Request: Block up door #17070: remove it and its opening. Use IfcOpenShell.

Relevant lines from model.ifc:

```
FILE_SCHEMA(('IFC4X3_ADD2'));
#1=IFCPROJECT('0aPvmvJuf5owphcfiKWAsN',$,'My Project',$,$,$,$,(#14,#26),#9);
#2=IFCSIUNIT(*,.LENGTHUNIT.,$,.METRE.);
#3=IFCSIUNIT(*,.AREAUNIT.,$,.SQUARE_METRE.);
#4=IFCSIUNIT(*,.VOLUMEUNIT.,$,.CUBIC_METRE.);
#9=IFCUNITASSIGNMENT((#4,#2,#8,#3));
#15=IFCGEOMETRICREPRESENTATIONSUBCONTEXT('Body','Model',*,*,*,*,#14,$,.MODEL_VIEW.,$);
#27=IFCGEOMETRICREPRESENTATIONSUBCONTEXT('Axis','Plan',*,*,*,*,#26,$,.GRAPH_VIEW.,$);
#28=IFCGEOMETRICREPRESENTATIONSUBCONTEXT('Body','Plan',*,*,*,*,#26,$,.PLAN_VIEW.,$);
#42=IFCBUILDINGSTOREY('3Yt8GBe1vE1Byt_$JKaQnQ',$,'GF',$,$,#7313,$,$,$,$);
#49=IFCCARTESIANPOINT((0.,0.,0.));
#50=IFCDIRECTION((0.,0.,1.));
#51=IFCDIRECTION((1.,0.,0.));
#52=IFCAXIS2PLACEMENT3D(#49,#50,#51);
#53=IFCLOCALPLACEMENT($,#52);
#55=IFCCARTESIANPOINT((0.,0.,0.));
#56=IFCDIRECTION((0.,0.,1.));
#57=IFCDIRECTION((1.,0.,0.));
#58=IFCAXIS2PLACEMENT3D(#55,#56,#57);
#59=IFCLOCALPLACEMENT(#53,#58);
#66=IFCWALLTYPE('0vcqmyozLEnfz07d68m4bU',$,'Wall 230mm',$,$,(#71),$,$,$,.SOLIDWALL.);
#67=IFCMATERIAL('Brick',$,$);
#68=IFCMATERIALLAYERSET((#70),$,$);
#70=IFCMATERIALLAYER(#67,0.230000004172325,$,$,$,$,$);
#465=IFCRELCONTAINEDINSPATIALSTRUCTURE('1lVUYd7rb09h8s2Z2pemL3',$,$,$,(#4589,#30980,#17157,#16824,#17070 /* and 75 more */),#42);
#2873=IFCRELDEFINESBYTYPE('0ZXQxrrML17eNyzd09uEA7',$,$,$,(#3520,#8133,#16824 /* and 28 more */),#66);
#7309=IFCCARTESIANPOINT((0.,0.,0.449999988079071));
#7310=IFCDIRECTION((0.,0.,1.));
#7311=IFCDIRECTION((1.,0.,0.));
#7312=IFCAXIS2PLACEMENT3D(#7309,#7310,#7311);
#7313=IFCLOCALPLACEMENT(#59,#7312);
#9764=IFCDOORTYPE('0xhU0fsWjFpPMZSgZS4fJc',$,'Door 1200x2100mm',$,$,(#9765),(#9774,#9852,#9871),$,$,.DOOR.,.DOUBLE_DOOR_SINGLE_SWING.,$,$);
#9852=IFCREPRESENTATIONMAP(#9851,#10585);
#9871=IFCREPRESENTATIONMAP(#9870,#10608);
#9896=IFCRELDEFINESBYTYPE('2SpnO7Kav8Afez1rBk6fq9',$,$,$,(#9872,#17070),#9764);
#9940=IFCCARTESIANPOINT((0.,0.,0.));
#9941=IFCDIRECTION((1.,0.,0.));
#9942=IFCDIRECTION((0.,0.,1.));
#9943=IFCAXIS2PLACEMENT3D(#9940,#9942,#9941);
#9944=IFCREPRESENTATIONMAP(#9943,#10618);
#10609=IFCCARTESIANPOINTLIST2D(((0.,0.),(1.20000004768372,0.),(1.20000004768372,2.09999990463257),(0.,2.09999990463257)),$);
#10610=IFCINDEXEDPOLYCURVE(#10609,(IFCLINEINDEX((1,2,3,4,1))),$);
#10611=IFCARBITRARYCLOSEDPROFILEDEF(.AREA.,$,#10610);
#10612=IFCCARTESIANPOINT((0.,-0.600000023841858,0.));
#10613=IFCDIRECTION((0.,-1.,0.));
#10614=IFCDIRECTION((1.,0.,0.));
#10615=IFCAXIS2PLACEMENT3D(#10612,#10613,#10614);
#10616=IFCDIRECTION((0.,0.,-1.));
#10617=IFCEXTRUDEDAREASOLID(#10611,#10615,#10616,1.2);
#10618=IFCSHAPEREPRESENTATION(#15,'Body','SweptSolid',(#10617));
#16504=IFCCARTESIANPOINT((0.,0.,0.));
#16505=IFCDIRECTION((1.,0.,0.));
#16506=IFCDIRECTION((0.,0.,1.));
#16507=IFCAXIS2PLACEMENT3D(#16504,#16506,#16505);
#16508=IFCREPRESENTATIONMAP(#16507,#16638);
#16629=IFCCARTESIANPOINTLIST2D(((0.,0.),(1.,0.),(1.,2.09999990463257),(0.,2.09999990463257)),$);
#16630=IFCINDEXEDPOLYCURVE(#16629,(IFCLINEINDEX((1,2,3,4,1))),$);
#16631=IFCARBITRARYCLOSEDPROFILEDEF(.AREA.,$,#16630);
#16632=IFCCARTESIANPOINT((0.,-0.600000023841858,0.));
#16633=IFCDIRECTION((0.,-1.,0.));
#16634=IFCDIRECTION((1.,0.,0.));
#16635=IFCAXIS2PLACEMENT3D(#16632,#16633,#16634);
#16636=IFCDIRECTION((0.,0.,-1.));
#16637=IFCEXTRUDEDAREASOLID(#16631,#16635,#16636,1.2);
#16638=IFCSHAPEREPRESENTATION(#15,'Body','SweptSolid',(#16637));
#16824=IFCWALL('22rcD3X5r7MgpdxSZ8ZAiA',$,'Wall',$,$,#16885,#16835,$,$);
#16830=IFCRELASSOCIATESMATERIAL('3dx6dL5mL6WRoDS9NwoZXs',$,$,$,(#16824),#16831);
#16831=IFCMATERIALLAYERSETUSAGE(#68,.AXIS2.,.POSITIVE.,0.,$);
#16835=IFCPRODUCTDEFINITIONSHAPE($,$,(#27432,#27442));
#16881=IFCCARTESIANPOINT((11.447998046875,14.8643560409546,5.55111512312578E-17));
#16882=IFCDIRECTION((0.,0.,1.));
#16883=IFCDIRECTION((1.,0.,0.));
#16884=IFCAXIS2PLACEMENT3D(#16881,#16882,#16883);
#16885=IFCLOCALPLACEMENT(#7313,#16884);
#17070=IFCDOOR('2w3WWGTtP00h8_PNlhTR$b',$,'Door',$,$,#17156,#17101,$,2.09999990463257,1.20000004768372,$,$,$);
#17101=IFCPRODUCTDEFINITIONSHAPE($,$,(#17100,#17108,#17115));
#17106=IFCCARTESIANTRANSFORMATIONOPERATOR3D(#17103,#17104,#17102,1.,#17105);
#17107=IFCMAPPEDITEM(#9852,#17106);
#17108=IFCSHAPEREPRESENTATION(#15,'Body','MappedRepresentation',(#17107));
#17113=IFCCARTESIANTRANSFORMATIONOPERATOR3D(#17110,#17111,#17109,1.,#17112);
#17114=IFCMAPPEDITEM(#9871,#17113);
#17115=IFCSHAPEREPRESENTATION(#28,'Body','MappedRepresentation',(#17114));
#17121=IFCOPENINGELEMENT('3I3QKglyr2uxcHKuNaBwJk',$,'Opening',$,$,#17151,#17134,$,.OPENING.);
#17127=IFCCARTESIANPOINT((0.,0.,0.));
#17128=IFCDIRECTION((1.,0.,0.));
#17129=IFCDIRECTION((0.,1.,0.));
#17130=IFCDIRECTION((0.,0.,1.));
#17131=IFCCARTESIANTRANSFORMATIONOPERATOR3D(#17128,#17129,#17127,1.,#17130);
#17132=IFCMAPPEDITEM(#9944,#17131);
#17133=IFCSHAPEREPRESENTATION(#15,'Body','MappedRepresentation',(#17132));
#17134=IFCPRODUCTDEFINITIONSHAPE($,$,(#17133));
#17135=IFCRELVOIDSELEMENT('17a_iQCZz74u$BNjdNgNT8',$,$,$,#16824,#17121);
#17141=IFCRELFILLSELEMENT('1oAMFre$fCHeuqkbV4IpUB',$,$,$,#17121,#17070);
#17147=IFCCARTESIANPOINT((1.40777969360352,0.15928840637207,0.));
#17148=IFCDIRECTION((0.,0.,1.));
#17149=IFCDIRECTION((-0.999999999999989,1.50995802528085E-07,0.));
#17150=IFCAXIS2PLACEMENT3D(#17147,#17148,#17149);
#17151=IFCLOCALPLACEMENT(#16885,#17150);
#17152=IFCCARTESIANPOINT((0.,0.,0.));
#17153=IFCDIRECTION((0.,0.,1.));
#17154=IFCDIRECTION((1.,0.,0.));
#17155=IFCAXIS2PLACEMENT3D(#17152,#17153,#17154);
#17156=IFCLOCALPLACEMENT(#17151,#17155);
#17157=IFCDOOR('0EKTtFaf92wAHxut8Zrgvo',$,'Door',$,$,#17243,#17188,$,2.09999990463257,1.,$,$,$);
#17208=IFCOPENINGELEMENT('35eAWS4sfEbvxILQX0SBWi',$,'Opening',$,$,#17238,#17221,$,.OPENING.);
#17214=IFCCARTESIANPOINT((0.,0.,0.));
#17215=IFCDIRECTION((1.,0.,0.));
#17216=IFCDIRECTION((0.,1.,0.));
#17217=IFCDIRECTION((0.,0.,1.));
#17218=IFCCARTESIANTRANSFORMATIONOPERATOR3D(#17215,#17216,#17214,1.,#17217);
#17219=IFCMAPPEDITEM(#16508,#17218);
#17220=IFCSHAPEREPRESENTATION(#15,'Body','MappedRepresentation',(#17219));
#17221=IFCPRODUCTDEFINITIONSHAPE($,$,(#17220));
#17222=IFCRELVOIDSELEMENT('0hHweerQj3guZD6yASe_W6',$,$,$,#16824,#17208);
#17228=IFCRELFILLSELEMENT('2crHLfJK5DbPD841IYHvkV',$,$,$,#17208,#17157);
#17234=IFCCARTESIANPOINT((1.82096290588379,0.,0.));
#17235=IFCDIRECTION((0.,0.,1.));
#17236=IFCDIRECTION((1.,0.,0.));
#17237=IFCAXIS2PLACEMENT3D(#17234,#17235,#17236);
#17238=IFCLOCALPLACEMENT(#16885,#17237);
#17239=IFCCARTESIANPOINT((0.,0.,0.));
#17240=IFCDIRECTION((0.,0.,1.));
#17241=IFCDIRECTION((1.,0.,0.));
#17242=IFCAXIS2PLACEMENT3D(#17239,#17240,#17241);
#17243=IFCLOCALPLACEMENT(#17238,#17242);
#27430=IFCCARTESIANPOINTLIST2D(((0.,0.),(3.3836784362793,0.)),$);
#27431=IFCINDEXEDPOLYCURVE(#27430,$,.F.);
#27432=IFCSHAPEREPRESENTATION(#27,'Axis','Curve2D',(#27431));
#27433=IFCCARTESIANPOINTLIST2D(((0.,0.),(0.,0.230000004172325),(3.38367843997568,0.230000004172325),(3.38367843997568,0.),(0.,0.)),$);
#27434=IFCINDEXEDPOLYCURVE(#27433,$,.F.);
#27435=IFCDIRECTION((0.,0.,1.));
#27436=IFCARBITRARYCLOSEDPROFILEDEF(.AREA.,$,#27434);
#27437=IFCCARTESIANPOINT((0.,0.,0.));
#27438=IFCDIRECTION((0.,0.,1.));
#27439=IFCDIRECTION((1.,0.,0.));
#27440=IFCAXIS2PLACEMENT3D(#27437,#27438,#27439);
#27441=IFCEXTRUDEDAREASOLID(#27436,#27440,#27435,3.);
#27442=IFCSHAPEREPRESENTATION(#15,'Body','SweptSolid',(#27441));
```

```python
import ifcopenshell
import ifcopenshell.api.feature
import ifcopenshell.api.root
import ifcopenshell.geom
import ifcopenshell.util.shape

model = ifcopenshell.open("model.ifc")
settings = ifcopenshell.geom.settings()


def volume(element):
    """Net volume in cubic metres, openings subtracted."""
    shape = ifcopenshell.geom.create_shape(settings, element)
    return ifcopenshell.util.shape.get_volume(shape.geometry)


door = model.by_guid("2w3WWGTtP00h8_PNlhTR$b")
opening = door.FillsVoids[0].RelatingOpeningElement
wall = opening.VoidsElements[0].RelatingBuildingElement
before = volume(wall)

ifcopenshell.api.root.remove_product(model, product=door)
ifcopenshell.api.feature.remove_feature(model, feature=opening)

after = volume(wall)

print(f"wall volume {before:.3f} -> {after:.3f} m3")

model.write("model_v2.ifc")
```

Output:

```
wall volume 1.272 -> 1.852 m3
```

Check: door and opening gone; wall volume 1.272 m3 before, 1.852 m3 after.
